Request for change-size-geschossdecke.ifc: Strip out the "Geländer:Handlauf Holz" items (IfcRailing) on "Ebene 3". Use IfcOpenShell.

First a look at what the model holds.

```python
import ifcopenshell
import ifcopenshell.util.element

model = ifcopenshell.open("change-size-geschossdecke.ifc")
print(model.schema)
storey = next(s for s in model.by_type("IfcBuildingStorey") if s.Name == "Ebene 3")
railings = [e for e in ifcopenshell.util.element.get_decomposition(storey) if e.is_a("IfcRailing")]
seen = {}
for e in railings:
    element_type = ifcopenshell.util.element.get_type(e)
    name = element_type.Name if element_type not in (None, e) else None
    seen[name] = seen.get(name, 0) + 1
for name, count in sorted(seen.items(), key=str):
    print(count, "x", name)
```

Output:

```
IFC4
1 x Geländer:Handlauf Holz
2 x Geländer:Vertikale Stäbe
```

```python
import ifcopenshell
import ifcopenshell.api.root
import ifcopenshell.util.element

model = ifcopenshell.open("change-size-geschossdecke.ifc")

storey = next(s for s in model.by_type("IfcBuildingStorey") if s.Name == "Ebene 3")
railings = [e for e in ifcopenshell.util.element.get_decomposition(storey) if e.is_a("IfcRailing")]
targets = [e for e in railings if (t := ifcopenshell.util.element.get_type(e)) not in (None, e) and t.Name == "Geländer:Handlauf Holz"]

for e in targets:
    ifcopenshell.api.root.remove_product(model, product=e)
print(len(targets), "removed")

model.write("change-size-geschossdecke_v2.ifc")
```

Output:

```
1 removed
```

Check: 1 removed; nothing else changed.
